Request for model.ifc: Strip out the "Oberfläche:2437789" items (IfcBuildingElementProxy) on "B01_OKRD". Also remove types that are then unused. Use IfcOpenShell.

First a look at what the model holds.

```python
import ifcopenshell
import ifcopenshell.util.element

model = ifcopenshell.open("model.ifc")
print(model.schema)
storey = next(s for s in model.by_type("IfcBuildingStorey") if s.Name == "B01_OKRD")
proxies = [e for e in ifcopenshell.util.element.get_decomposition(storey) if e.is_a("IfcBuildingElementProxy")]
seen = {}
for e in proxies:
    element_type = ifcopenshell.util.element.get_type(e)
    name = element_type.Name if element_type not in (None, e) else None
    seen[name] = seen.get(name, 0) + 1
for name, count in sorted(seen.items(), key=str):
    print(count, "x", name)
```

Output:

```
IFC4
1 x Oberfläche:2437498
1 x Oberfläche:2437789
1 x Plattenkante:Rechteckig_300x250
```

```python
import ifcopenshell
import ifcopenshell.api.root
import ifcopenshell.util.element

model = ifcopenshell.open("model.ifc")

storey = next(s for s in model.by_type("IfcBuildingStorey") if s.Name == "B01_OKRD")
proxies = [e for e in ifcopenshell.util.element.get_decomposition(storey) if e.is_a("IfcBuildingElementProxy")]
targets = [e for e in proxies if (t := ifcopenshell.util.element.get_type(e)) not in (None, e) and t.Name == "Oberfläche:2437789"]
types = {ifcopenshell.util.element.get_type(e) for e in targets} - {None, *targets}

for e in targets:
    ifcopenshell.api.root.remove_product(model, product=e)
print(len(targets), "removed")

unused = [t for t in types if not ifcopenshell.util.element.get_types(t)]
for t in unused:
    ifcopenshell.api.root.remove_product(model, product=t)
print(len(unused), "unused types removed")

model.write("model_edited.ifc")
```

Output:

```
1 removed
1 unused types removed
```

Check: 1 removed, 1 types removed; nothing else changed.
